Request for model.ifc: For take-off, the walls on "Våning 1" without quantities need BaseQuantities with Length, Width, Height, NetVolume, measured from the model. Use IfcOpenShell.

First a look at what the model holds.

```python
import ifcopenshell
import ifcopenshell.util.element
import ifcopenshell.util.unit

model = ifcopenshell.open("model.ifc")
print(model.schema)
for unit_type in ("LENGTHUNIT", "AREAUNIT", "VOLUMEUNIT"):
    print(unit_type, ifcopenshell.util.unit.calculate_unit_scale(model, unit_type))
storey = next(s for s in model.by_type("IfcBuildingStorey") if s.Name == "Våning 1")
walls = [e for e in ifcopenshell.util.element.get_decomposition(storey) if e.is_a("IfcWall")]
for e in sorted(walls, key=lambda e: e.id()):
    print(e.id(), e.is_a(), e.Name, list(ifcopenshell.util.element.get_psets(e, qtos_only=True)), sep=" | ")
```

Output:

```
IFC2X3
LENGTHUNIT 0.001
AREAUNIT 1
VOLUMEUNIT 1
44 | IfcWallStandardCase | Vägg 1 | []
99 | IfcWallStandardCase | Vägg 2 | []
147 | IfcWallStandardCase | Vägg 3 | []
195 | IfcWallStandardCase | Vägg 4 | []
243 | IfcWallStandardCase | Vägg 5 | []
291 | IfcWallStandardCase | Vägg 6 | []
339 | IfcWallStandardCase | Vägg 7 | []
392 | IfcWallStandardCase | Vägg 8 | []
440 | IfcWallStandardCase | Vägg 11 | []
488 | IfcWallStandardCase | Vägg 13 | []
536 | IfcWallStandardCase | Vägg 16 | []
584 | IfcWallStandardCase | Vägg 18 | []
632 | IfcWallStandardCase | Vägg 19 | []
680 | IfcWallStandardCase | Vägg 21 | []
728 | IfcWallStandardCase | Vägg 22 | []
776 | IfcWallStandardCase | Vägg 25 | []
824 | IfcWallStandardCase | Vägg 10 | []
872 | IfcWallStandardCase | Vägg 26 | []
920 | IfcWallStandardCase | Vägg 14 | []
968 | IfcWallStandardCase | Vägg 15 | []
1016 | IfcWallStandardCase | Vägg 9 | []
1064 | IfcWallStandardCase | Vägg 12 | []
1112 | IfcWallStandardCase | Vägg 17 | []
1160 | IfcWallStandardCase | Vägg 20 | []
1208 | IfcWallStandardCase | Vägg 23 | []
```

```python
import ifcopenshell
import ifcopenshell.api.pset
import ifcopenshell.geom
import ifcopenshell.util.element
import ifcopenshell.util.shape
import ifcopenshell.util.unit

model = ifcopenshell.open("model.ifc")
unit_scale = ifcopenshell.util.unit.calculate_unit_scale(model)
volume_scale = ifcopenshell.util.unit.calculate_unit_scale(model, "VOLUMEUNIT")
settings = ifcopenshell.geom.settings()

storey = next(s for s in model.by_type("IfcBuildingStorey") if s.Name == "Våning 1")
walls = [e for e in ifcopenshell.util.element.get_decomposition(storey) if e.is_a("IfcWall")]

for e in sorted(walls, key=lambda e: e.id()):
    if ifcopenshell.util.element.get_psets(e, qtos_only=True, should_inherit=False):
        continue
    # Geometry comes back in metres, in the element's own axes.
    shape = ifcopenshell.geom.create_shape(settings, e)
    values = {
        "Length": ifcopenshell.util.shape.get_x(shape.geometry) / unit_scale,
        "Width": ifcopenshell.util.shape.get_y(shape.geometry) / unit_scale,
        "Height": ifcopenshell.util.shape.get_z(shape.geometry) / unit_scale,
        "NetVolume": ifcopenshell.util.shape.get_volume(shape.geometry) / volume_scale,
    }
    qto = ifcopenshell.api.pset.add_qto(model, product=e, name="BaseQuantities")
    ifcopenshell.api.pset.edit_qto(model, qto=qto, properties=values)
    print(e.id(), {k: round(v, 3) for k, v in values.items()})

model.write("model_v2.ifc")
```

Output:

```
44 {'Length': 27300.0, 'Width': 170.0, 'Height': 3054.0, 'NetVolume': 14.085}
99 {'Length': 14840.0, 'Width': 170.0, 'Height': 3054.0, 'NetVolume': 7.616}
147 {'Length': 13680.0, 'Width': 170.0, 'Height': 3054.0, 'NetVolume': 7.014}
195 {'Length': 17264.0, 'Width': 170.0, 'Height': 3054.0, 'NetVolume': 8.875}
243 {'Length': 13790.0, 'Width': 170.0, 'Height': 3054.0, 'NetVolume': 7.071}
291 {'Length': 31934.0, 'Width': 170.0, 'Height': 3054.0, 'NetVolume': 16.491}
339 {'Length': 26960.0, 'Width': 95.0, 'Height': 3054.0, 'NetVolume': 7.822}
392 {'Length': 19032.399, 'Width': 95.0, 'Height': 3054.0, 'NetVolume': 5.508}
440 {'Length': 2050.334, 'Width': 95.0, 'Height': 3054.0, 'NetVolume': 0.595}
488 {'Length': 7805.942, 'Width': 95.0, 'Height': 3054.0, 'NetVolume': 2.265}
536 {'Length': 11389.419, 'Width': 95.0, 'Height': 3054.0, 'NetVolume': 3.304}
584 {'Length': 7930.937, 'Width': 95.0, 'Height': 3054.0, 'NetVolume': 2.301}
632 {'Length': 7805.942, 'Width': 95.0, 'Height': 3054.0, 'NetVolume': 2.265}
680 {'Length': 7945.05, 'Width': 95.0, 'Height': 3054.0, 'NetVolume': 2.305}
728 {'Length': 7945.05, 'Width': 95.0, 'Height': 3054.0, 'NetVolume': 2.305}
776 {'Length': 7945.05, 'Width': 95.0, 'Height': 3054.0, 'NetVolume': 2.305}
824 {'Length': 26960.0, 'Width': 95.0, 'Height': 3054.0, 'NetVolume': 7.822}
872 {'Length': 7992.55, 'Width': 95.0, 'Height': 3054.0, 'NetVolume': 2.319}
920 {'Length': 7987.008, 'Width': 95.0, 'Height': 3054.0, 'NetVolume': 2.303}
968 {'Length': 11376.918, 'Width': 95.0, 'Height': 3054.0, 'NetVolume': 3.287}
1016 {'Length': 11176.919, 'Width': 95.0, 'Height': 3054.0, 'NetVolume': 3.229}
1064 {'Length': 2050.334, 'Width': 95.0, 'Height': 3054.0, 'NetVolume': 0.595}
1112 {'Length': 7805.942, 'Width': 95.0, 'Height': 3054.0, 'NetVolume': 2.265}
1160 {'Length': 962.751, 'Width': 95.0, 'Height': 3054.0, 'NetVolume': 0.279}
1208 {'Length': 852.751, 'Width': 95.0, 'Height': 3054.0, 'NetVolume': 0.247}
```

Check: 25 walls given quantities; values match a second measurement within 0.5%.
